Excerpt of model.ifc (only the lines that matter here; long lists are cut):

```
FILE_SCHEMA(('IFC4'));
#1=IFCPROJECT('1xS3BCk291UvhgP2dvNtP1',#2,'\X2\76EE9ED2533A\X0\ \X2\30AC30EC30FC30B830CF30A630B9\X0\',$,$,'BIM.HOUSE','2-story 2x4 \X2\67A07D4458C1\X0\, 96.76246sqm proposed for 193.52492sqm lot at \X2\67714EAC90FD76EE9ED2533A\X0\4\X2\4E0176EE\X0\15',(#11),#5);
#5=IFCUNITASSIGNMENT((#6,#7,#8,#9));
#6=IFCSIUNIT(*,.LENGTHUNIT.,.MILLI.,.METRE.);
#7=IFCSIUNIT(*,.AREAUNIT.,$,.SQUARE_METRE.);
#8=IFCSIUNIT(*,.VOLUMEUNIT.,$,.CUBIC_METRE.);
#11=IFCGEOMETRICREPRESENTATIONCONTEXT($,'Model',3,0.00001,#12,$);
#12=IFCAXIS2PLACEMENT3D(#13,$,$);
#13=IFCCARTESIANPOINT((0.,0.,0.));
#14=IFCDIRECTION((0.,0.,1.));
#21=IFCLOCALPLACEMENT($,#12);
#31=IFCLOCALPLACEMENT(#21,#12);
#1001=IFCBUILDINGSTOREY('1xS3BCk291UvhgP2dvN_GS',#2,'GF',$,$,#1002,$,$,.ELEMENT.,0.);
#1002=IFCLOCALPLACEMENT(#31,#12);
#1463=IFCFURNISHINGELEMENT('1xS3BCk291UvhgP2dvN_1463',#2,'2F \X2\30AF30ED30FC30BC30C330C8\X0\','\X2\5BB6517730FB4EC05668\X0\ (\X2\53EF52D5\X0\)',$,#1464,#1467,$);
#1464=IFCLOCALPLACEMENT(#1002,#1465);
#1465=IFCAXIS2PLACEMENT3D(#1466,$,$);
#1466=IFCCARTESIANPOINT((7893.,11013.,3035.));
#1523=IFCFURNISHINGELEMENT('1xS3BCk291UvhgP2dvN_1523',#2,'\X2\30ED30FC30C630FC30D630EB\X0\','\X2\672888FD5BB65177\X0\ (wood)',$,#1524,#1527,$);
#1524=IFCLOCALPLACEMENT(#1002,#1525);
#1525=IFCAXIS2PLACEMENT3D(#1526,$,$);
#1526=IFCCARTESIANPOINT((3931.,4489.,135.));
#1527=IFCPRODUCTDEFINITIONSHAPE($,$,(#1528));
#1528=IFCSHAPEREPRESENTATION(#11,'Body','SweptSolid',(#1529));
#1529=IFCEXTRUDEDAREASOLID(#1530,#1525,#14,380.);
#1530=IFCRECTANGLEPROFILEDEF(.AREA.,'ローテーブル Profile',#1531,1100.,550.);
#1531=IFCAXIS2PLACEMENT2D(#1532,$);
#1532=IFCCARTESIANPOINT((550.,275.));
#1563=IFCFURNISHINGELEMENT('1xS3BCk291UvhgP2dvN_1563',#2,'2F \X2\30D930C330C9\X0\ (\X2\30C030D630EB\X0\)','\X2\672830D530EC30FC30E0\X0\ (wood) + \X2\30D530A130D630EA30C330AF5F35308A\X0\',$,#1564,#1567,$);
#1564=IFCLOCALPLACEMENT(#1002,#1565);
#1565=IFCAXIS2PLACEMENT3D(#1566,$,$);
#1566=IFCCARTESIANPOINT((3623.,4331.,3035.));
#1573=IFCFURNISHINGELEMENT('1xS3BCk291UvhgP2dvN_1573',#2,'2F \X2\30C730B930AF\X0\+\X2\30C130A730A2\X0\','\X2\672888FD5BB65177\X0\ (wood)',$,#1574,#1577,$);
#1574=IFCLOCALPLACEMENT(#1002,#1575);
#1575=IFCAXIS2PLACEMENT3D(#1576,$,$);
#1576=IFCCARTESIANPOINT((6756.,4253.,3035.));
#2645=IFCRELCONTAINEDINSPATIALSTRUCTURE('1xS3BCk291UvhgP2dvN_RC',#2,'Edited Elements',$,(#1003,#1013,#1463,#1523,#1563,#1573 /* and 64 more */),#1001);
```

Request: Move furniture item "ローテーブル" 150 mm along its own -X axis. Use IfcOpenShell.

```python
import ifcopenshell
import ifcopenshell.api.geometry
import ifcopenshell.util.placement
import ifcopenshell.util.unit

model = ifcopenshell.open("model.ifc")
unit_scale = ifcopenshell.util.unit.calculate_unit_scale(model)

item = model.by_guid("1xS3BCk291UvhgP2dvN_1523")
matrix = ifcopenshell.util.placement.get_local_placement(item.ObjectPlacement)
matrix[:3, 3] -= matrix[:3, 0] * 0.15 / unit_scale
ifcopenshell.api.geometry.edit_object_placement(model, product=item, matrix=matrix, is_si=False)

print(ifcopenshell.util.placement.get_local_placement(item.ObjectPlacement).round(3) + 0.0)

model.write("model_v2.ifc")
```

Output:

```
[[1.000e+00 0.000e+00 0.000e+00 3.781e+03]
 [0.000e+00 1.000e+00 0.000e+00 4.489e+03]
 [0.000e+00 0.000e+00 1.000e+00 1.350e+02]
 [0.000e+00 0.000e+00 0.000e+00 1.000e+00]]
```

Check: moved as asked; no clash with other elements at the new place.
